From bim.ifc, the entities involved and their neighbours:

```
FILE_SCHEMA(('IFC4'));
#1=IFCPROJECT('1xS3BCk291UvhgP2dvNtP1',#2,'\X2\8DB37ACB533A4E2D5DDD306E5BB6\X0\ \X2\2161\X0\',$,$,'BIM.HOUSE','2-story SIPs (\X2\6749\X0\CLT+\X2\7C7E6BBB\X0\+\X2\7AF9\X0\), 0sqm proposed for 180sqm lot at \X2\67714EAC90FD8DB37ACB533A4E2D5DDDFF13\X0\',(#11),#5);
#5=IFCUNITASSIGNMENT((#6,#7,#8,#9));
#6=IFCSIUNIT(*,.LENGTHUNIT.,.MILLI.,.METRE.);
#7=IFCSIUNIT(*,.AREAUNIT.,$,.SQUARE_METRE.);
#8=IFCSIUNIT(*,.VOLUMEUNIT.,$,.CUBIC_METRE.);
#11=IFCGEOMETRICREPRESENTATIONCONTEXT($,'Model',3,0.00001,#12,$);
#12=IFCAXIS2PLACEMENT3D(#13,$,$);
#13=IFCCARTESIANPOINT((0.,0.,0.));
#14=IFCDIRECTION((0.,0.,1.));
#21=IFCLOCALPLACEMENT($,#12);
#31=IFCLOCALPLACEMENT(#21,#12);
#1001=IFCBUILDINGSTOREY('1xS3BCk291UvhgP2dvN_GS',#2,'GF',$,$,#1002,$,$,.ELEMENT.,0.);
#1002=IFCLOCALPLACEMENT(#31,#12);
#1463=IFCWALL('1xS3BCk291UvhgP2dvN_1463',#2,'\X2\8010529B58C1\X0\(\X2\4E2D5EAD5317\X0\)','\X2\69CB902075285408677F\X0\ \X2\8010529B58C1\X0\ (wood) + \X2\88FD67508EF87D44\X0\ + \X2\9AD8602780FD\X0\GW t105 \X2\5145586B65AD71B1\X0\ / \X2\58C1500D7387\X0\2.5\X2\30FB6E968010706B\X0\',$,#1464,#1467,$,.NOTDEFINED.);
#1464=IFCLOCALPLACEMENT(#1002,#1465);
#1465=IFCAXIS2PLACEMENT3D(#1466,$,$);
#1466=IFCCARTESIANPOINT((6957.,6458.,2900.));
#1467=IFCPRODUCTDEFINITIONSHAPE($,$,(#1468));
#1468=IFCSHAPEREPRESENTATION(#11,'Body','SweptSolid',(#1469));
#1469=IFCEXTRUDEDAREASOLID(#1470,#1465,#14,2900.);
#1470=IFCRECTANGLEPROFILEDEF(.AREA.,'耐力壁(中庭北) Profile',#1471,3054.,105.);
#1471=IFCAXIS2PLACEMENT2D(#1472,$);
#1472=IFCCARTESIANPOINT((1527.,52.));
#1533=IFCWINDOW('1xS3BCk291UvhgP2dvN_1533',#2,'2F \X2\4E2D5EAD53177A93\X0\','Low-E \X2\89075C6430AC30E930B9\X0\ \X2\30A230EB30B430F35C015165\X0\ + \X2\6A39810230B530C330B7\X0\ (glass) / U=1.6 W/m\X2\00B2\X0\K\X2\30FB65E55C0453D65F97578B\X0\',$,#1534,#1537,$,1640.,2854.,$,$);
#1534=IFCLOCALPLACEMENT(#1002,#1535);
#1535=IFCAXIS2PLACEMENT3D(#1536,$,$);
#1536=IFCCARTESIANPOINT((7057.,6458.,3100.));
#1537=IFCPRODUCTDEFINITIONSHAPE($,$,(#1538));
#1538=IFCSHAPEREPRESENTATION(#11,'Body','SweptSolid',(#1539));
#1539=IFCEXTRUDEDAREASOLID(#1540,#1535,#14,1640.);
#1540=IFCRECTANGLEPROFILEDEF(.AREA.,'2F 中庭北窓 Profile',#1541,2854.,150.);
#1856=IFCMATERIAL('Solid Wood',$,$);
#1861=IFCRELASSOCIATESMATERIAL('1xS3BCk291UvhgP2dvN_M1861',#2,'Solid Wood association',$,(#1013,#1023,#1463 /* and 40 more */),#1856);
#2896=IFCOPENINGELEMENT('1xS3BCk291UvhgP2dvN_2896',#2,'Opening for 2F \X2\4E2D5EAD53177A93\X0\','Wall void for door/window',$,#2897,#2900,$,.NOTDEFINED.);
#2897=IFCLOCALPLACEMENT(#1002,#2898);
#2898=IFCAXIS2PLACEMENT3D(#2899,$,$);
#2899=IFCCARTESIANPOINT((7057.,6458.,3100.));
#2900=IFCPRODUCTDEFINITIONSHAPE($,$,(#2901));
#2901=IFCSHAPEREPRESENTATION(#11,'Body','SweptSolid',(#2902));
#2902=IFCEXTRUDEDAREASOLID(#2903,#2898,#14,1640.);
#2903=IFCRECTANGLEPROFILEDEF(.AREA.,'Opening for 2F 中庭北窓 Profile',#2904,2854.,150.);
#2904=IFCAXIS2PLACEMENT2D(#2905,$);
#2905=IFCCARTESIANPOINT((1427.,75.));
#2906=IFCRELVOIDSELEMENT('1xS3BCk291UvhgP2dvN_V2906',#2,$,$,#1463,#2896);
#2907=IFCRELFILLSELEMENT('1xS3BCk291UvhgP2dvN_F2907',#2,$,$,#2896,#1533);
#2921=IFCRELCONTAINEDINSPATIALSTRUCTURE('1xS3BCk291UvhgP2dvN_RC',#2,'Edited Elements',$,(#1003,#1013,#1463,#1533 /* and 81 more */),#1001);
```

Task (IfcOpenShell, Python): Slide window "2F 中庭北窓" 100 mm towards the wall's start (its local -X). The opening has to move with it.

```python
import ifcopenshell
import ifcopenshell.api.geometry
import ifcopenshell.util.placement
import ifcopenshell.util.unit

model = ifcopenshell.open("bim.ifc")
unit_scale = ifcopenshell.util.unit.calculate_unit_scale(model)

window = model.by_guid("1xS3BCk291UvhgP2dvN_1533")
opening = window.FillsVoids[0].RelatingOpeningElement
wall = opening.VoidsElements[0].RelatingBuildingElement

wall_matrix = ifcopenshell.util.placement.get_local_placement(wall.ObjectPlacement)
shift = wall_matrix[:3, 0] * -0.1 / unit_scale
before = ifcopenshell.util.placement.get_local_placement(window.ObjectPlacement)[:3, 3].copy()

# The window is not placed relative to its opening, so move both.
for product in (opening, window):
    matrix = ifcopenshell.util.placement.get_local_placement(product.ObjectPlacement)
    matrix[:3, 3] += shift
    ifcopenshell.api.geometry.edit_object_placement(model, product=product, matrix=matrix, is_si=False)

after = ifcopenshell.util.placement.get_local_placement(window.ObjectPlacement)[:3, 3]
print("window moved by", (after - before).round(3) + 0.0)

model.write("bim_v2.ifc")
```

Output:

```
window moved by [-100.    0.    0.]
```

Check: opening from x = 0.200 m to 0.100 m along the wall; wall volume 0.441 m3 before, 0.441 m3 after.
